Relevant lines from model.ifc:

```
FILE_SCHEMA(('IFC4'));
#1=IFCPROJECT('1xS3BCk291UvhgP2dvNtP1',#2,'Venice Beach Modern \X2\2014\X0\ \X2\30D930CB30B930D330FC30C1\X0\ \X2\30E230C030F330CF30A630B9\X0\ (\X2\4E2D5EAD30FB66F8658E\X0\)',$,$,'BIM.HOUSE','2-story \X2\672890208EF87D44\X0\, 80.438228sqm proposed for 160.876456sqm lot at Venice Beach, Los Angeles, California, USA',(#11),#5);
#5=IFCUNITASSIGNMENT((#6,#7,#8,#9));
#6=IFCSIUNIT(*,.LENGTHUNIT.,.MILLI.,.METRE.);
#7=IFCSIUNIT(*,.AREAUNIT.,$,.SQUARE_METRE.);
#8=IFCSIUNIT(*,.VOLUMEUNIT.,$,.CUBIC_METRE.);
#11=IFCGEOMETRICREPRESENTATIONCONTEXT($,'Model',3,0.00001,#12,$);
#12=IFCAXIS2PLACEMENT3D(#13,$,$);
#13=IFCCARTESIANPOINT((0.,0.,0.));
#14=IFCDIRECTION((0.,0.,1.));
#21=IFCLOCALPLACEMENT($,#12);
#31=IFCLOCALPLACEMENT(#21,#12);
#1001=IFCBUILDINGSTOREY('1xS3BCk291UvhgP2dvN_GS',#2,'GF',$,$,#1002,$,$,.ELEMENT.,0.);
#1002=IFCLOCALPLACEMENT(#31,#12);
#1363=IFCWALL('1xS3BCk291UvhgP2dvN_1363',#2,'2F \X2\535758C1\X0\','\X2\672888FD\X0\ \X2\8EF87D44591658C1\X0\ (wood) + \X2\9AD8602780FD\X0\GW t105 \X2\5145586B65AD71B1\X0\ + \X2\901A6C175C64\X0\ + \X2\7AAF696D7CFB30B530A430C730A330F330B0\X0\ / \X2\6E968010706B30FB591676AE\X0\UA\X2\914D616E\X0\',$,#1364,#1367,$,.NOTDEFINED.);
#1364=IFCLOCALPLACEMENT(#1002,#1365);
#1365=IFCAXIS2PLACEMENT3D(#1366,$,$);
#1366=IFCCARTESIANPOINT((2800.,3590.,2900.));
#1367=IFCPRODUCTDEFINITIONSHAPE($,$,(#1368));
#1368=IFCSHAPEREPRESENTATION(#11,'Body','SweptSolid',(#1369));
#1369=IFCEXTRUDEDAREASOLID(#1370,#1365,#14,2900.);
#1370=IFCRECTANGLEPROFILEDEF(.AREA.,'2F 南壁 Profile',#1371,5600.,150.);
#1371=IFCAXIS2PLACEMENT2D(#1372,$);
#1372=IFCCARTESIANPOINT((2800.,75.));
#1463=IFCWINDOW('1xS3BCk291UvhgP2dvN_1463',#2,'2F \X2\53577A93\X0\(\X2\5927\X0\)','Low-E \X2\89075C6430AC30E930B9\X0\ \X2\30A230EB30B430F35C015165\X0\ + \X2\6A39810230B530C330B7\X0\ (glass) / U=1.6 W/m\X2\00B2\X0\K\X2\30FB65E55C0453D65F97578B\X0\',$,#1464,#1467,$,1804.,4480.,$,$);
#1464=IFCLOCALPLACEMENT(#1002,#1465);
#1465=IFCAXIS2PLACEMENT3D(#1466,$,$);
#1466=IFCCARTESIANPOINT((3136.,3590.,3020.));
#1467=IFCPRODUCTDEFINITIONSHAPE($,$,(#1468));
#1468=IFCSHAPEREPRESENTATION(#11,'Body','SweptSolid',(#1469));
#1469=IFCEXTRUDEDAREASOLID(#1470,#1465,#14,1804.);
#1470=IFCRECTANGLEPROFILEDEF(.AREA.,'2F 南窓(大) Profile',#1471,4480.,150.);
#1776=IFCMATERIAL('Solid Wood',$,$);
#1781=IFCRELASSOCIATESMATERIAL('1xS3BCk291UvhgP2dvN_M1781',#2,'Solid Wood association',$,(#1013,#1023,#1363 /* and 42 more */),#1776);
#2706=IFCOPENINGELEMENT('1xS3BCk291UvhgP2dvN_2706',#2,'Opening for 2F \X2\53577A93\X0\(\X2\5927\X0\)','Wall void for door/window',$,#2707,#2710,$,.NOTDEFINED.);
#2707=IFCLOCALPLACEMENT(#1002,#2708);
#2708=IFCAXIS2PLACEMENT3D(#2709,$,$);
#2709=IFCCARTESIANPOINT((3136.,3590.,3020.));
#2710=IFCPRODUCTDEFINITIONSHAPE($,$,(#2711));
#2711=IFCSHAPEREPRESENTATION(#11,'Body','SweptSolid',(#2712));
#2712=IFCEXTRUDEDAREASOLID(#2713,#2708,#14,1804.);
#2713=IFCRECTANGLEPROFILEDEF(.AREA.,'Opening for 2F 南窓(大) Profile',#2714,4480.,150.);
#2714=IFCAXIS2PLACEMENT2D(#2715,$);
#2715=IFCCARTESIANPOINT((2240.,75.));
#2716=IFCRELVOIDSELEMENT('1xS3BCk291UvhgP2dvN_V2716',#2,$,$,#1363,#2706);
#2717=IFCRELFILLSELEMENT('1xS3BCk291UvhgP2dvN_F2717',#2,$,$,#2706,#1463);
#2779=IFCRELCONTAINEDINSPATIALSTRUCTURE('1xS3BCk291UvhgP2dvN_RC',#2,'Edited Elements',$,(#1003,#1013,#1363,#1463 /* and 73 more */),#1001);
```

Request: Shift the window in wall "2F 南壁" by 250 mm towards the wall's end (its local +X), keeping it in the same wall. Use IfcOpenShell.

```python
import ifcopenshell
import ifcopenshell.api.geometry
import ifcopenshell.util.placement

model = ifcopenshell.open("model.ifc")

window = model.by_id(1463)
opening = window.FillsVoids[0].RelatingOpeningElement
wall = opening.VoidsElements[0].RelatingBuildingElement

wall_matrix = ifcopenshell.util.placement.get_local_placement(wall.ObjectPlacement)
shift = wall_matrix[:3, 0] * 250.0
before = ifcopenshell.util.placement.get_local_placement(window.ObjectPlacement)[:3, 3].copy()

# The window is not placed relative to its opening, so move both.
for product in (opening, window):
    matrix = ifcopenshell.util.placement.get_local_placement(product.ObjectPlacement)
    matrix[:3, 3] += shift
    ifcopenshell.api.geometry.edit_object_placement(model, product=product, matrix=matrix, is_si=False)

after = ifcopenshell.util.placement.get_local_placement(window.ObjectPlacement)[:3, 3]
print("window moved by", (after - before).round(3) + 0.0)

model.write("model_edited.ifc")
```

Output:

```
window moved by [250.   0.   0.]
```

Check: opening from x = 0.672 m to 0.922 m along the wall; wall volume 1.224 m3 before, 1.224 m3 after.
